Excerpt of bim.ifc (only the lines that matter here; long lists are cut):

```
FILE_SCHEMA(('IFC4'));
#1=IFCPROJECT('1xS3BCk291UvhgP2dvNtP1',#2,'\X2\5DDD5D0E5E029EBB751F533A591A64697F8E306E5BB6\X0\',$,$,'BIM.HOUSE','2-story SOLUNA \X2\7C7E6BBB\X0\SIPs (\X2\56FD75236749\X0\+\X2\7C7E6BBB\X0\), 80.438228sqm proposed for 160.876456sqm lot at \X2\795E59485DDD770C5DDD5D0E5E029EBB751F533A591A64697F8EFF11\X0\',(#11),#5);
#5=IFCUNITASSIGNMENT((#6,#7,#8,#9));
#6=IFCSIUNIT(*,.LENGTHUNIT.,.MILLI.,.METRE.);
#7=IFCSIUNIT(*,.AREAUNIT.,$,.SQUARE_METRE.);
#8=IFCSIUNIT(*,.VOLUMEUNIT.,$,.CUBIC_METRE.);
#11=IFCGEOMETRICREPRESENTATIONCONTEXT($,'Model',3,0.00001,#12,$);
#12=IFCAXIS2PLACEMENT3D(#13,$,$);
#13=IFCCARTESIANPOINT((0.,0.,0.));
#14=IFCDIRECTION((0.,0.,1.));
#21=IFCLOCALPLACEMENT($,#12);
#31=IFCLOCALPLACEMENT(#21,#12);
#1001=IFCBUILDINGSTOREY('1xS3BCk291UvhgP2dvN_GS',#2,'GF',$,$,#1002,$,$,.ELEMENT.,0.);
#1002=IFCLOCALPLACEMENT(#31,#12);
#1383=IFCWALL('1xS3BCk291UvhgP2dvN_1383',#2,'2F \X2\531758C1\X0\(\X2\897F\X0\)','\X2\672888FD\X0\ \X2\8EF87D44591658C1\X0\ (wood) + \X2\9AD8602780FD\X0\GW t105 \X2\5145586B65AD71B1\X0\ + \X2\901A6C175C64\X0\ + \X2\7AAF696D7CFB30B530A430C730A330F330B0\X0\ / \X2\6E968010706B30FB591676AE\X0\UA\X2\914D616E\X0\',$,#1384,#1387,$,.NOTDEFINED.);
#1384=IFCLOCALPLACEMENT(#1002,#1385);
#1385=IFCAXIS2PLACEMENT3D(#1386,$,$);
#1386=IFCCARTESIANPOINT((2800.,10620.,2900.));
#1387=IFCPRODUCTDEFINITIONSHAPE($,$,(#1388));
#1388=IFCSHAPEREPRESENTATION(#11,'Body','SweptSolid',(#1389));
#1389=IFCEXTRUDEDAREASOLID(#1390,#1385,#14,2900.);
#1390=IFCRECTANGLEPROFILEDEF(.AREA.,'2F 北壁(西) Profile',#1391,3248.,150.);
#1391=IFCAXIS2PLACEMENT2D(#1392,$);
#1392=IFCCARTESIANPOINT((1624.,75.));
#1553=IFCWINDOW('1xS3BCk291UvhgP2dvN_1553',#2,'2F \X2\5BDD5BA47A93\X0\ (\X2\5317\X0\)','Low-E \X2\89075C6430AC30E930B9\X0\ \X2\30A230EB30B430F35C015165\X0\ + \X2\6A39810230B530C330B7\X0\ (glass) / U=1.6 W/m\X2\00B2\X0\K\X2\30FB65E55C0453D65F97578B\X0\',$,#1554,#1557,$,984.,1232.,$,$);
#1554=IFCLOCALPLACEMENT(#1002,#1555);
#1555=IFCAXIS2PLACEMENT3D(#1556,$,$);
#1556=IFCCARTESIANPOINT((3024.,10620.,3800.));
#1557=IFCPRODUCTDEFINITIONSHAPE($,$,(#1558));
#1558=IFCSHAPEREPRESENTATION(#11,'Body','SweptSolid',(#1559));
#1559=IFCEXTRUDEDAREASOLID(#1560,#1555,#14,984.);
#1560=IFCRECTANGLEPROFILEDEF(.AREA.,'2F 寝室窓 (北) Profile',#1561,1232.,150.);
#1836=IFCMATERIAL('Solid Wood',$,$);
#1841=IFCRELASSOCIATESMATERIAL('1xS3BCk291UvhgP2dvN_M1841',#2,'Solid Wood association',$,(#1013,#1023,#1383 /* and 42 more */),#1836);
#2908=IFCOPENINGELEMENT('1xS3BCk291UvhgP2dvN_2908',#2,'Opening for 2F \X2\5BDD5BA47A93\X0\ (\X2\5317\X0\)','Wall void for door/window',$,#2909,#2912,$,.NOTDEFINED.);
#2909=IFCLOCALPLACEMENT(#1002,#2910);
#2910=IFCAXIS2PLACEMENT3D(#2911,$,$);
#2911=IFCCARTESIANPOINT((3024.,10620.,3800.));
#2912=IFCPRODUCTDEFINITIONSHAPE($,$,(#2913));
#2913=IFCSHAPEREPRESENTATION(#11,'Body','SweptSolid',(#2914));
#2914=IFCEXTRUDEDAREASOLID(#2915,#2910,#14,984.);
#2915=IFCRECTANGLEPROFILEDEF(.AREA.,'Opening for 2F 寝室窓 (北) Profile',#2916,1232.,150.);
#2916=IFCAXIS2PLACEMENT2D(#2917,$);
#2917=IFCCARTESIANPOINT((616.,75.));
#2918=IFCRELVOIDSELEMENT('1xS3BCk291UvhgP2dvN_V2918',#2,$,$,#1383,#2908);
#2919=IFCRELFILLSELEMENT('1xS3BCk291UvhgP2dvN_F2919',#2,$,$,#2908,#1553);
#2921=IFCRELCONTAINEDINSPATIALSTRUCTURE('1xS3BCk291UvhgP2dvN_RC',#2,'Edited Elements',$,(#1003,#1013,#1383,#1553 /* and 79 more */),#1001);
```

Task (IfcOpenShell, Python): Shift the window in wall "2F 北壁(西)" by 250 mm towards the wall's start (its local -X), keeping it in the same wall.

```python
import ifcopenshell
import ifcopenshell.api.geometry
import ifcopenshell.util.placement

model = ifcopenshell.open("bim.ifc")

window = model.by_guid("1xS3BCk291UvhgP2dvN_1553")
opening = window.FillsVoids[0].RelatingOpeningElement
wall = opening.VoidsElements[0].RelatingBuildingElement

wall_matrix = ifcopenshell.util.placement.get_local_placement(wall.ObjectPlacement)
shift = wall_matrix[:3, 0] * -250.0
before = ifcopenshell.util.placement.get_local_placement(window.ObjectPlacement)[:3, 3].copy()

# The window is not placed relative to its opening, so move both.
for product in (opening, window):
    matrix = ifcopenshell.util.placement.get_local_placement(product.ObjectPlacement)
    matrix[:3, 3] += shift
    ifcopenshell.api.geometry.edit_object_placement(model, product=product, matrix=matrix, is_si=False)

after = ifcopenshell.util.placement.get_local_placement(window.ObjectPlacement)[:3, 3]
print("window moved by", (after - before).round(3) + 0.0)

model.write("bim-out.ifc")
```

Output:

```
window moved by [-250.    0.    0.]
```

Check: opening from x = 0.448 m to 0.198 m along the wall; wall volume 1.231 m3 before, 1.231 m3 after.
